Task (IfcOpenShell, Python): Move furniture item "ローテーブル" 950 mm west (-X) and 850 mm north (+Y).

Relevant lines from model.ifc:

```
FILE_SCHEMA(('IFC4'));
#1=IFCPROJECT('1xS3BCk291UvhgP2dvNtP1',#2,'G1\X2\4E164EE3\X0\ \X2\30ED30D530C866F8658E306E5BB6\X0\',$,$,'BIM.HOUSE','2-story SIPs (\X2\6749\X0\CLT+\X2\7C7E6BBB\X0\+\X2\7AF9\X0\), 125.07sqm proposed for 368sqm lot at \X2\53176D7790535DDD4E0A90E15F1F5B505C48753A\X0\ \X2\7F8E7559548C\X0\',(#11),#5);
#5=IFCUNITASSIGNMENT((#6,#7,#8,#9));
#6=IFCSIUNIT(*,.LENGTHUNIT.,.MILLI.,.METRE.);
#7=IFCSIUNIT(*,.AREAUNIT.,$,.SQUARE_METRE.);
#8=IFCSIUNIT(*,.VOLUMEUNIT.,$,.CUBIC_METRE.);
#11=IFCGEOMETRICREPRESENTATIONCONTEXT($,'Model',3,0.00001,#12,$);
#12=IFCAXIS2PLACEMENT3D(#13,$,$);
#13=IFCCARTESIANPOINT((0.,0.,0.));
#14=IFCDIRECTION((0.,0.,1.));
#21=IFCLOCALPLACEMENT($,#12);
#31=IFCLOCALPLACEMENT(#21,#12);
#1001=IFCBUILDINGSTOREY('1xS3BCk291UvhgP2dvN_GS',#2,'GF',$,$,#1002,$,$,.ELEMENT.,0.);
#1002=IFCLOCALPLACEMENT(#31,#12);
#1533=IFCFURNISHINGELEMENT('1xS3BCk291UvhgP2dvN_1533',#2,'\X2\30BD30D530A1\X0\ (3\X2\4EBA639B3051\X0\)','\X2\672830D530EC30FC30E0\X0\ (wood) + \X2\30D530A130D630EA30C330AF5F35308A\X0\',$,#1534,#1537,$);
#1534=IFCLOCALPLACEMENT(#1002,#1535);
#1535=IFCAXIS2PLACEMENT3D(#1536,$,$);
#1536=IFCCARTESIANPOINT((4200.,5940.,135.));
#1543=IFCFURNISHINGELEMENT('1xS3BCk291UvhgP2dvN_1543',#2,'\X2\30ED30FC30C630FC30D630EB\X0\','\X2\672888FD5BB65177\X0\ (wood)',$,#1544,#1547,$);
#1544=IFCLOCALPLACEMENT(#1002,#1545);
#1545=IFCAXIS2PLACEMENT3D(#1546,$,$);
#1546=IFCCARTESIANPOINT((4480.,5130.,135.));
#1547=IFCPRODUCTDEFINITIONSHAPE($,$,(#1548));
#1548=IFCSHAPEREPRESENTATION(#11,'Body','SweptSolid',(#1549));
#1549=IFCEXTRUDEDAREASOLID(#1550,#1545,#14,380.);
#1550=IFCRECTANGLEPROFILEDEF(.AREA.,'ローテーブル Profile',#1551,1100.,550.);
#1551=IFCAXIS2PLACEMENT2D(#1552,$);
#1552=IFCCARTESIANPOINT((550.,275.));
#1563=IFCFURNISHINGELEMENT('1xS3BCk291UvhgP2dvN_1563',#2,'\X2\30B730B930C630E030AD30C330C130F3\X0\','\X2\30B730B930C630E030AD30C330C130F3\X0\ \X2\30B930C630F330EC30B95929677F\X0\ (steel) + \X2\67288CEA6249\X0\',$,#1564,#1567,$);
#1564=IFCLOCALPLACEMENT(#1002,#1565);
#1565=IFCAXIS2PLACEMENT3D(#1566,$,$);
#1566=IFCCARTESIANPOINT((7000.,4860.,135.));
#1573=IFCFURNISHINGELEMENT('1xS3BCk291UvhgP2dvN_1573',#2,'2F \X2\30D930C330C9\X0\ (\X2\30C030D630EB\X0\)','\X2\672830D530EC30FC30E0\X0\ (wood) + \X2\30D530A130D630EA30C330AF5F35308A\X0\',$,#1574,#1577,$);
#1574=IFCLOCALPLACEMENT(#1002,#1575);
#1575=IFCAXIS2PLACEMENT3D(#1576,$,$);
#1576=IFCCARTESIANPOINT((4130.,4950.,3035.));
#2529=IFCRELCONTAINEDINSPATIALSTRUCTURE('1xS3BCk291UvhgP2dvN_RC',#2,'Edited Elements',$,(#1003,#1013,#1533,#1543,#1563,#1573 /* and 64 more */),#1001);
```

```python
import ifcopenshell
import ifcopenshell.api.geometry
import ifcopenshell.util.placement
import ifcopenshell.util.unit

model = ifcopenshell.open("model.ifc")
unit_scale = ifcopenshell.util.unit.calculate_unit_scale(model)

item = model.by_id(1543)
matrix = ifcopenshell.util.placement.get_local_placement(item.ObjectPlacement)
matrix[0, 3] -= 0.95 / unit_scale
matrix[1, 3] += 0.85 / unit_scale
ifcopenshell.api.geometry.edit_object_placement(model, product=item, matrix=matrix, is_si=False)

print(ifcopenshell.util.placement.get_local_placement(item.ObjectPlacement).round(3) + 0.0)

model.write("model_edited.ifc")
```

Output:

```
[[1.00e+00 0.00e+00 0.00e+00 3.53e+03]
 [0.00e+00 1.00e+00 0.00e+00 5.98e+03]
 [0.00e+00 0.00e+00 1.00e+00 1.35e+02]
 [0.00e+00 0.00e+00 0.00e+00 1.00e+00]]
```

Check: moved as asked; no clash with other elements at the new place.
